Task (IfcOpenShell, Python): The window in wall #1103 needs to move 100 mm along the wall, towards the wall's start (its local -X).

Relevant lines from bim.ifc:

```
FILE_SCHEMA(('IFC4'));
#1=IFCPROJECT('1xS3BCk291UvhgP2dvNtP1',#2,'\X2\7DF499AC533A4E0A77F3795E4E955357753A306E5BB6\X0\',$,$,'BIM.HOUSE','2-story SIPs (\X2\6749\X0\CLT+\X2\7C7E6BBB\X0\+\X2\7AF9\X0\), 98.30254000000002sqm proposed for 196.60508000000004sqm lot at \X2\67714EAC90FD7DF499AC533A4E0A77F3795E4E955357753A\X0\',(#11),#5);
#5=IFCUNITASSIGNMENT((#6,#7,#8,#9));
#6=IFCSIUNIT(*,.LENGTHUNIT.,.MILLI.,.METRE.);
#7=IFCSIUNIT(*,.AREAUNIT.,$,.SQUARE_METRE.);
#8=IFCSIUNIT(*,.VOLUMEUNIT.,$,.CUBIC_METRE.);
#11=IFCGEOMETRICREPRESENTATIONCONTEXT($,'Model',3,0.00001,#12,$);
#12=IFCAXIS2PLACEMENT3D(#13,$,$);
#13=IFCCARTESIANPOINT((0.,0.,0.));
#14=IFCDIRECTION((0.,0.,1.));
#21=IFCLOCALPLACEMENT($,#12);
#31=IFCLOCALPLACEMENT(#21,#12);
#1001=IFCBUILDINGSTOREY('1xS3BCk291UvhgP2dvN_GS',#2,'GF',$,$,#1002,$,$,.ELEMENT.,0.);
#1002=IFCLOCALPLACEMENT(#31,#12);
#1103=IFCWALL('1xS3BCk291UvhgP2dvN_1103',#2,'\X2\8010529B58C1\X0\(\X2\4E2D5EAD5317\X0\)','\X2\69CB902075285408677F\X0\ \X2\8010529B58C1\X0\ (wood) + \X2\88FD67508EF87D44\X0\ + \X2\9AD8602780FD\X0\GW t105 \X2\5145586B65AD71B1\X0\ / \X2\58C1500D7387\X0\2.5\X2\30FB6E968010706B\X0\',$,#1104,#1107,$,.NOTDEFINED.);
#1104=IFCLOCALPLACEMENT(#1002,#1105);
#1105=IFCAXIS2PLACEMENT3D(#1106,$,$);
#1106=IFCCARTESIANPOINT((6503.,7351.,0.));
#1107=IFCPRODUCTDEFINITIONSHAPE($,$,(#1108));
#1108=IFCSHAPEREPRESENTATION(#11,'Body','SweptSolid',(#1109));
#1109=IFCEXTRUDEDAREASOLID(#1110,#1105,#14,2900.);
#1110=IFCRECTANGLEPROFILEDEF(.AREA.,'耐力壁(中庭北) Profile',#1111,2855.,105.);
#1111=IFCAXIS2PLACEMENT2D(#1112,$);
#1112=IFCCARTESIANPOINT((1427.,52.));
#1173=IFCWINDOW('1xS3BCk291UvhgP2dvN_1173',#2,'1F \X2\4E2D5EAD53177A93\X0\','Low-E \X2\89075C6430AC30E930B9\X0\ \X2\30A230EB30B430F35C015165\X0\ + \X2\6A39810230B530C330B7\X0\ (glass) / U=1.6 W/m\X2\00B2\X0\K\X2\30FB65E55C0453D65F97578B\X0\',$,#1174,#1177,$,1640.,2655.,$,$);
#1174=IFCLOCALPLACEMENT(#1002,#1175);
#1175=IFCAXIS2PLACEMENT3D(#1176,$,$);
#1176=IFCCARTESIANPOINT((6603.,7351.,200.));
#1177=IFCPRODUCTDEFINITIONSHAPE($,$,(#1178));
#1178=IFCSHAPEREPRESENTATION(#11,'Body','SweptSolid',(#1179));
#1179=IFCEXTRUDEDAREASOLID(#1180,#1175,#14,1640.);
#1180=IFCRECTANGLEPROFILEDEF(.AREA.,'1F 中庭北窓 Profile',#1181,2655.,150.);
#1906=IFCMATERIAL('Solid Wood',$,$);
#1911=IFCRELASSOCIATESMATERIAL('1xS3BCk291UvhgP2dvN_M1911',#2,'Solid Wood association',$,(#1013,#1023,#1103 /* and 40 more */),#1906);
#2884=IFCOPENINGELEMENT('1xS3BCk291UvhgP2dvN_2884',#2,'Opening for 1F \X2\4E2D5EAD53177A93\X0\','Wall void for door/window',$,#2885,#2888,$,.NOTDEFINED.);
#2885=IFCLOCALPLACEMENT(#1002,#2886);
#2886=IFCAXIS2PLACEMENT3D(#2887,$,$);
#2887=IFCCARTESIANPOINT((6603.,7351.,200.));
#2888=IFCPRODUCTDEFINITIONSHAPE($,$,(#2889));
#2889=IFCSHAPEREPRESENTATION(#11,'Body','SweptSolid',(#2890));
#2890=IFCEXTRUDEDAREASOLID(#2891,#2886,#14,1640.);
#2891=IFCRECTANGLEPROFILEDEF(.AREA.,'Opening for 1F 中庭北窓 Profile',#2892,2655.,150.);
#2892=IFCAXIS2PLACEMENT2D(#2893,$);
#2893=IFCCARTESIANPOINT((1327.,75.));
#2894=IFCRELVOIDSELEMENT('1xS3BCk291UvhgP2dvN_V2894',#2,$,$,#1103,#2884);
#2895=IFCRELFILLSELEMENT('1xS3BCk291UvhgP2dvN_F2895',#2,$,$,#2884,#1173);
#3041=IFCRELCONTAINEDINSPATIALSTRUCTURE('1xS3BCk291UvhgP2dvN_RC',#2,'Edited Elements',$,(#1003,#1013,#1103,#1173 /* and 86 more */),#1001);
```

```python
import ifcopenshell
import ifcopenshell.api.geometry
import ifcopenshell.util.placement
import ifcopenshell.util.unit

model = ifcopenshell.open("bim.ifc")
unit_scale = ifcopenshell.util.unit.calculate_unit_scale(model)

window = model.by_guid("1xS3BCk291UvhgP2dvN_1173")
opening = window.FillsVoids[0].RelatingOpeningElement
wall = opening.VoidsElements[0].RelatingBuildingElement

wall_matrix = ifcopenshell.util.placement.get_local_placement(wall.ObjectPlacement)
shift = wall_matrix[:3, 0] * -0.1 / unit_scale
before = ifcopenshell.util.placement.get_local_placement(window.ObjectPlacement)[:3, 3].copy()

# The window is not placed relative to its opening, so move both.
for product in (opening, window):
    matrix = ifcopenshell.util.placement.get_local_placement(product.ObjectPlacement)
    matrix[:3, 3] += shift
    ifcopenshell.api.geometry.edit_object_placement(model, product=product, matrix=matrix, is_si=False)

after = ifcopenshell.util.placement.get_local_placement(window.ObjectPlacement)[:3, 3]
print("window moved by", (after - before).round(3) + 0.0)

model.write("bim_rev.ifc")
```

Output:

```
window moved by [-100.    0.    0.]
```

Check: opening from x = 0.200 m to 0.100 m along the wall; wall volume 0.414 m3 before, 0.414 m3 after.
